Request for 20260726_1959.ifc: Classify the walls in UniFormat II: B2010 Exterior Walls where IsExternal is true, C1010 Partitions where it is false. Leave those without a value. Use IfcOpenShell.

First a look at what the model holds.

```python
import ifcopenshell
import ifcopenshell.util.element

model = ifcopenshell.open("20260726_1959.ifc")
print(model.schema)
print("classifications:", [c.Name for c in model.by_type("IfcClassification")])
values = [ifcopenshell.util.element.get_pset(e, "Pset_WallCommon", "IsExternal") for e in model.by_type("IfcWall")]
for value in (True, False, None):
    print("IsExternal", value, values.count(value))
```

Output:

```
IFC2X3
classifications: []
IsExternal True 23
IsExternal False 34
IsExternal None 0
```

```python
import ifcopenshell
import ifcopenshell.api.classification
import ifcopenshell.util.element

model = ifcopenshell.open("20260726_1959.ifc")

# IFC2X3 requires Source and Edition and has no link from the project to the system.
system = model.create_entity("IfcClassification", Source="ASTM", Edition="E1557", Name="UniFormat II")

walls = model.by_type("IfcWall")
external = {e: ifcopenshell.util.element.get_pset(e, "Pset_WallCommon", "IsExternal") for e in walls}
for flag, code, name in ((True, "B2010", "Exterior Walls"), (False, "C1010", "Partitions")):
    products = [e for e in walls if external[e] is flag]
    ifcopenshell.api.classification.add_reference(
        model, products=products, classification=system, identification=code, name=name
    )
    print(code, len(products))

model.write("20260726_1959-out.ifc")
```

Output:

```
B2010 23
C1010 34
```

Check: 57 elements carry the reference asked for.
